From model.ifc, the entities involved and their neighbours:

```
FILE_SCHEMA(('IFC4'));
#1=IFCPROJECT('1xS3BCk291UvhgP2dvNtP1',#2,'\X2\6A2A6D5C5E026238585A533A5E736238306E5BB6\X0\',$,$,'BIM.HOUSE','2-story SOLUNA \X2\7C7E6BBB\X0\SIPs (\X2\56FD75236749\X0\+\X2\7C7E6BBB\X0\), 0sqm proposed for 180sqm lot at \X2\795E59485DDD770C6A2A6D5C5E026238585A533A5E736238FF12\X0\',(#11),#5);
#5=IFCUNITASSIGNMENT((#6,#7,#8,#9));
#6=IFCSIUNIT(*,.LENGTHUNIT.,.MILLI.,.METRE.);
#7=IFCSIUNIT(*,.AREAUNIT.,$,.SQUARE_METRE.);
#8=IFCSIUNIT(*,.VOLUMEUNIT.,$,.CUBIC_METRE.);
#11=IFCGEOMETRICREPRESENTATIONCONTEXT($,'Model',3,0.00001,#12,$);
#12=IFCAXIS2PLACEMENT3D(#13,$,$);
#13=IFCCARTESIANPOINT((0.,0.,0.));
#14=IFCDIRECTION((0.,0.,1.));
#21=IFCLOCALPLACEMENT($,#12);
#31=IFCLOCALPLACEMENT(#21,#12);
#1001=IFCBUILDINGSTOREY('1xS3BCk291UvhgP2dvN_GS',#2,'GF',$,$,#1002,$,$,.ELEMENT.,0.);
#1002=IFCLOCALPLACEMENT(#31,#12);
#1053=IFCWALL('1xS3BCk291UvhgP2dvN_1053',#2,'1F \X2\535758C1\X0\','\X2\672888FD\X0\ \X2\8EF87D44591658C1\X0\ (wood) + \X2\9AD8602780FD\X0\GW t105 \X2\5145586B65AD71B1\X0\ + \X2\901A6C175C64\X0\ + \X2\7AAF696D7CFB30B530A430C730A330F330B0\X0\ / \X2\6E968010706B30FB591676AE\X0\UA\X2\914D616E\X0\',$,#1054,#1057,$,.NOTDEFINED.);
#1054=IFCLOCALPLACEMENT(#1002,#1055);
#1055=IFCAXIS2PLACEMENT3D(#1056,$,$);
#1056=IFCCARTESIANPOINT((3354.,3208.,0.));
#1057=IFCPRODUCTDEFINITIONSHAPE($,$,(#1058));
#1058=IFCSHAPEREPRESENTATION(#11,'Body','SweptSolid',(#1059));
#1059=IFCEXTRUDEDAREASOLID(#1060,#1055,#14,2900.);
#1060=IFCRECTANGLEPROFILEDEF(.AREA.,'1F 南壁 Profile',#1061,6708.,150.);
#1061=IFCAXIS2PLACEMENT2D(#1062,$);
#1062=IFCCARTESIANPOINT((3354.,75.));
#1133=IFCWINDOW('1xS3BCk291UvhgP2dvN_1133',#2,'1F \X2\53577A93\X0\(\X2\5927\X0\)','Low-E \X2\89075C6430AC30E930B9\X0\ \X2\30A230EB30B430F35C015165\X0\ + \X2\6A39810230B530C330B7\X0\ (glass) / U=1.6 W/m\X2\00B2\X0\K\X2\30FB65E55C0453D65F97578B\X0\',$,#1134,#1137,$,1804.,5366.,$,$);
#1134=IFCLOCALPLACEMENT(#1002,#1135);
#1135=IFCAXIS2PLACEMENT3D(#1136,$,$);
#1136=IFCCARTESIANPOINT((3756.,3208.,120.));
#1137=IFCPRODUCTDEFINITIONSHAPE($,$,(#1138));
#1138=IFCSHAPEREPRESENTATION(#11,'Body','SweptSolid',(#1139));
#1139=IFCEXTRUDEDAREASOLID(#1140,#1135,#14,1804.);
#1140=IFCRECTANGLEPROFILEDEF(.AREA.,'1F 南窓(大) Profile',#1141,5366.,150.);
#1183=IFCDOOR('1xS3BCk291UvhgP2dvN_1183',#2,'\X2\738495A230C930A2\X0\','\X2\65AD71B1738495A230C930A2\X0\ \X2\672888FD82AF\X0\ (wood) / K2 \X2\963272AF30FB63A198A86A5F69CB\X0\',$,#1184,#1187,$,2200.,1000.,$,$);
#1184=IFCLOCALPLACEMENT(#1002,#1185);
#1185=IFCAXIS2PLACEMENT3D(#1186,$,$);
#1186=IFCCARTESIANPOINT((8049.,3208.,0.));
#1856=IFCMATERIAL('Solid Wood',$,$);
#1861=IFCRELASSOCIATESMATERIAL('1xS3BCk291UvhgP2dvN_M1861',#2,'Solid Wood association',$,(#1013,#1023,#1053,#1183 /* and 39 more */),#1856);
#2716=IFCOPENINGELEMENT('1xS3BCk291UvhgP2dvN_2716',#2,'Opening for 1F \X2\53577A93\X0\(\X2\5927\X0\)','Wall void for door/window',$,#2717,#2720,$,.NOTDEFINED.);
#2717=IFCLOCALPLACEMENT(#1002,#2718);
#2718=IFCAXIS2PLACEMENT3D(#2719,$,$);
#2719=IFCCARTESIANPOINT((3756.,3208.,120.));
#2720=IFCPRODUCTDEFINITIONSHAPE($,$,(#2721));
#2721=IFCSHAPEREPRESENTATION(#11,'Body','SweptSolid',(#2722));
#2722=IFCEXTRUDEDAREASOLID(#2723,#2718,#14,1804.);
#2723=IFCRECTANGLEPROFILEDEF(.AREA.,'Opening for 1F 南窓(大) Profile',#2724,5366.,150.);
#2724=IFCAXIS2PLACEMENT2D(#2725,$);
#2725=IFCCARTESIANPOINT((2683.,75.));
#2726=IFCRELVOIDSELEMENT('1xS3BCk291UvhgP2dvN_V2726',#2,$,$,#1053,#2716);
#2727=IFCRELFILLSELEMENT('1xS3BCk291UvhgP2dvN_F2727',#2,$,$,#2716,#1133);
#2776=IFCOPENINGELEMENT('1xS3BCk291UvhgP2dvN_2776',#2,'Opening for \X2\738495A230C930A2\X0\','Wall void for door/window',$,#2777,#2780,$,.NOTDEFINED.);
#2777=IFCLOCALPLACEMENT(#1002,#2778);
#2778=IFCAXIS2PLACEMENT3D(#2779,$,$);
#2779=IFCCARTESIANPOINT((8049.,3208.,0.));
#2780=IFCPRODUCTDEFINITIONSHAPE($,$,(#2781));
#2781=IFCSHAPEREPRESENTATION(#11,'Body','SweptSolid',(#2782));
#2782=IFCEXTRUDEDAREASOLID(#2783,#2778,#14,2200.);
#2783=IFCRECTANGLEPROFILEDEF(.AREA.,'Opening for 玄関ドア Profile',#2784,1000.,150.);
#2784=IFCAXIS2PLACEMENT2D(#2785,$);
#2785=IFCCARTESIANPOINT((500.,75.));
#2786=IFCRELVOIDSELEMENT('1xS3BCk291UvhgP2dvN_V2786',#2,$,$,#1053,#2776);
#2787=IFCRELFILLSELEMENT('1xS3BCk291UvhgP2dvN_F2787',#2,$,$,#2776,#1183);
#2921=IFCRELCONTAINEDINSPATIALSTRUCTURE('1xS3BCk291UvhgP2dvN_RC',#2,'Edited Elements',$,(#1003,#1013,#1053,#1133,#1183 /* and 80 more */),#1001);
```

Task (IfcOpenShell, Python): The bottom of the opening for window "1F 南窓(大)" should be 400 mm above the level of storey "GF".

```python
import numpy as np
import ifcopenshell
import ifcopenshell.api.geometry
import ifcopenshell.geom
import ifcopenshell.util.element
import ifcopenshell.util.placement
import ifcopenshell.util.shape
import ifcopenshell.util.unit

model = ifcopenshell.open("model.ifc")
unit_scale = ifcopenshell.util.unit.calculate_unit_scale(model)

window = model.by_guid("1xS3BCk291UvhgP2dvN_1133")
opening = window.FillsVoids[0].RelatingOpeningElement
storey = ifcopenshell.util.element.get_container(window, ifc_class="IfcBuildingStorey")
level = ifcopenshell.util.placement.get_local_placement(storey.ObjectPlacement)[2, 3]

# The opening's origin need not be at the sill, so measure its lowest point.
shape = ifcopenshell.geom.create_shape(ifcopenshell.geom.settings(), opening)
bottom = ifcopenshell.util.shape.get_shape_bottom_elevation(shape, shape.geometry) / unit_scale
dz = level + 0.4 / unit_scale - bottom

shift = np.array([0.0, 0.0, dz])
# The window is not placed relative to its opening, so move both.
for product in (opening, window):
    matrix = ifcopenshell.util.placement.get_local_placement(product.ObjectPlacement)
    matrix[:3, 3] += shift
    ifcopenshell.api.geometry.edit_object_placement(model, product=product, matrix=matrix, is_si=False)

print(f"moved by {dz * unit_scale:+.3f} m")

model.write("model-out.ifc")
```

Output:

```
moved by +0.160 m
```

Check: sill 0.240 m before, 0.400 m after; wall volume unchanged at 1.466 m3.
